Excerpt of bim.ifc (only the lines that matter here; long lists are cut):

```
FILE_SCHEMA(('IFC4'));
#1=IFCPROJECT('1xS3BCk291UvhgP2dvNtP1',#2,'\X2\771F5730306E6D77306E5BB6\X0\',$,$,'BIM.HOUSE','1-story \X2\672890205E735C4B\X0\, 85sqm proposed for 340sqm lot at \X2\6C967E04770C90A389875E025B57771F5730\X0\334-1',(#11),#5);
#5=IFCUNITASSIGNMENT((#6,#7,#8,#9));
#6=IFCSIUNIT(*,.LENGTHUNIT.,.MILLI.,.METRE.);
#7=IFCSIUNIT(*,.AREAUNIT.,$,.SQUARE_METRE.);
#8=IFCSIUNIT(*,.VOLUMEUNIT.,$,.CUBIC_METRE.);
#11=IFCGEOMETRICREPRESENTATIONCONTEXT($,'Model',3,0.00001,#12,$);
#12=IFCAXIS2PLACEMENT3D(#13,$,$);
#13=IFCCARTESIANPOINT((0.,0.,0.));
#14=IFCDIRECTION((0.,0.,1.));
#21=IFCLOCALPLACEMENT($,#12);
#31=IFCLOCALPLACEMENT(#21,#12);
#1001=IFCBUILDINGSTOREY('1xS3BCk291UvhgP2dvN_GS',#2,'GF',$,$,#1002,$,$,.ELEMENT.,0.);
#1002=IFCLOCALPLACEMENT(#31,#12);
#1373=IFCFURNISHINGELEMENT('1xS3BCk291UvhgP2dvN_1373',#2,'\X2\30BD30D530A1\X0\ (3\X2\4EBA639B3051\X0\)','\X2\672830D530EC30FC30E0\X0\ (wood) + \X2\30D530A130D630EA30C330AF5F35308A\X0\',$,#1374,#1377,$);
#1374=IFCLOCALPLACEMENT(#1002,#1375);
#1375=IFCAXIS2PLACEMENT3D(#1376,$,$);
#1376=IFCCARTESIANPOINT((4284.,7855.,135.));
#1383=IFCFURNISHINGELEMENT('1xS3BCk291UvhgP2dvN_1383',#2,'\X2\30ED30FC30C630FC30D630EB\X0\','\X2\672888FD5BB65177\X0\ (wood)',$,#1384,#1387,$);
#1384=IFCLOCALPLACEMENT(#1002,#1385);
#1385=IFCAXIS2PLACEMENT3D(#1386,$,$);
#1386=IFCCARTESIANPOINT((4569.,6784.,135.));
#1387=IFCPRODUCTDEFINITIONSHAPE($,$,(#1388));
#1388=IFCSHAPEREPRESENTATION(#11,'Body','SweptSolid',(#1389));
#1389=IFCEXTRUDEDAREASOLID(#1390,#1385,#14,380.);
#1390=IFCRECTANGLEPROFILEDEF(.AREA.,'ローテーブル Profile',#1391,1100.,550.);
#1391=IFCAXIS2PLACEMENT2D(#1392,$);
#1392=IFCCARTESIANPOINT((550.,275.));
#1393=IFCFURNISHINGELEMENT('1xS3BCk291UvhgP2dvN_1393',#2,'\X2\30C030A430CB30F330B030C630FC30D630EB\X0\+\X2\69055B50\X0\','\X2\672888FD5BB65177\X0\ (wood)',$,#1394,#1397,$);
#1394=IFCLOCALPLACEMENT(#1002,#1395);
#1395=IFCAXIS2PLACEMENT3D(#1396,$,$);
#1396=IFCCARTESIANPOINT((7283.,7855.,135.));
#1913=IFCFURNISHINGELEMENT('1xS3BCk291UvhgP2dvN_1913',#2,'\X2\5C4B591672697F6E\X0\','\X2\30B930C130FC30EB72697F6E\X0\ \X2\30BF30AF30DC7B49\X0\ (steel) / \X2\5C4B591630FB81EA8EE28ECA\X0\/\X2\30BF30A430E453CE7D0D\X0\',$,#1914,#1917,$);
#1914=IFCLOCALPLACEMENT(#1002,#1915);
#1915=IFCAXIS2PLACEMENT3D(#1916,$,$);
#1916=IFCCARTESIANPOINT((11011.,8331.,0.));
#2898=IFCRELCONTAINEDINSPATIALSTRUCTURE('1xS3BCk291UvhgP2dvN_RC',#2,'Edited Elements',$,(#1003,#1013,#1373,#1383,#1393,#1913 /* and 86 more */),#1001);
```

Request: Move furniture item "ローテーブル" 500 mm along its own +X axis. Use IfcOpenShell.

```python
import ifcopenshell
import ifcopenshell.api.geometry
import ifcopenshell.util.placement
import ifcopenshell.util.unit

model = ifcopenshell.open("bim.ifc")
unit_scale = ifcopenshell.util.unit.calculate_unit_scale(model)

item = model.by_guid("1xS3BCk291UvhgP2dvN_1383")
matrix = ifcopenshell.util.placement.get_local_placement(item.ObjectPlacement)
matrix[:3, 3] += matrix[:3, 0] * 0.5 / unit_scale
ifcopenshell.api.geometry.edit_object_placement(model, product=item, matrix=matrix, is_si=False)

print(ifcopenshell.util.placement.get_local_placement(item.ObjectPlacement).round(3) + 0.0)

model.write("bim-out.ifc")
```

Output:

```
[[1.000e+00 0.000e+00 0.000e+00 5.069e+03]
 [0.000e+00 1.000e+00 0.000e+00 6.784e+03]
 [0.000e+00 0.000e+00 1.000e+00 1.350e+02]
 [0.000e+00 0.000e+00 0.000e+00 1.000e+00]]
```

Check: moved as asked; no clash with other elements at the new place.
